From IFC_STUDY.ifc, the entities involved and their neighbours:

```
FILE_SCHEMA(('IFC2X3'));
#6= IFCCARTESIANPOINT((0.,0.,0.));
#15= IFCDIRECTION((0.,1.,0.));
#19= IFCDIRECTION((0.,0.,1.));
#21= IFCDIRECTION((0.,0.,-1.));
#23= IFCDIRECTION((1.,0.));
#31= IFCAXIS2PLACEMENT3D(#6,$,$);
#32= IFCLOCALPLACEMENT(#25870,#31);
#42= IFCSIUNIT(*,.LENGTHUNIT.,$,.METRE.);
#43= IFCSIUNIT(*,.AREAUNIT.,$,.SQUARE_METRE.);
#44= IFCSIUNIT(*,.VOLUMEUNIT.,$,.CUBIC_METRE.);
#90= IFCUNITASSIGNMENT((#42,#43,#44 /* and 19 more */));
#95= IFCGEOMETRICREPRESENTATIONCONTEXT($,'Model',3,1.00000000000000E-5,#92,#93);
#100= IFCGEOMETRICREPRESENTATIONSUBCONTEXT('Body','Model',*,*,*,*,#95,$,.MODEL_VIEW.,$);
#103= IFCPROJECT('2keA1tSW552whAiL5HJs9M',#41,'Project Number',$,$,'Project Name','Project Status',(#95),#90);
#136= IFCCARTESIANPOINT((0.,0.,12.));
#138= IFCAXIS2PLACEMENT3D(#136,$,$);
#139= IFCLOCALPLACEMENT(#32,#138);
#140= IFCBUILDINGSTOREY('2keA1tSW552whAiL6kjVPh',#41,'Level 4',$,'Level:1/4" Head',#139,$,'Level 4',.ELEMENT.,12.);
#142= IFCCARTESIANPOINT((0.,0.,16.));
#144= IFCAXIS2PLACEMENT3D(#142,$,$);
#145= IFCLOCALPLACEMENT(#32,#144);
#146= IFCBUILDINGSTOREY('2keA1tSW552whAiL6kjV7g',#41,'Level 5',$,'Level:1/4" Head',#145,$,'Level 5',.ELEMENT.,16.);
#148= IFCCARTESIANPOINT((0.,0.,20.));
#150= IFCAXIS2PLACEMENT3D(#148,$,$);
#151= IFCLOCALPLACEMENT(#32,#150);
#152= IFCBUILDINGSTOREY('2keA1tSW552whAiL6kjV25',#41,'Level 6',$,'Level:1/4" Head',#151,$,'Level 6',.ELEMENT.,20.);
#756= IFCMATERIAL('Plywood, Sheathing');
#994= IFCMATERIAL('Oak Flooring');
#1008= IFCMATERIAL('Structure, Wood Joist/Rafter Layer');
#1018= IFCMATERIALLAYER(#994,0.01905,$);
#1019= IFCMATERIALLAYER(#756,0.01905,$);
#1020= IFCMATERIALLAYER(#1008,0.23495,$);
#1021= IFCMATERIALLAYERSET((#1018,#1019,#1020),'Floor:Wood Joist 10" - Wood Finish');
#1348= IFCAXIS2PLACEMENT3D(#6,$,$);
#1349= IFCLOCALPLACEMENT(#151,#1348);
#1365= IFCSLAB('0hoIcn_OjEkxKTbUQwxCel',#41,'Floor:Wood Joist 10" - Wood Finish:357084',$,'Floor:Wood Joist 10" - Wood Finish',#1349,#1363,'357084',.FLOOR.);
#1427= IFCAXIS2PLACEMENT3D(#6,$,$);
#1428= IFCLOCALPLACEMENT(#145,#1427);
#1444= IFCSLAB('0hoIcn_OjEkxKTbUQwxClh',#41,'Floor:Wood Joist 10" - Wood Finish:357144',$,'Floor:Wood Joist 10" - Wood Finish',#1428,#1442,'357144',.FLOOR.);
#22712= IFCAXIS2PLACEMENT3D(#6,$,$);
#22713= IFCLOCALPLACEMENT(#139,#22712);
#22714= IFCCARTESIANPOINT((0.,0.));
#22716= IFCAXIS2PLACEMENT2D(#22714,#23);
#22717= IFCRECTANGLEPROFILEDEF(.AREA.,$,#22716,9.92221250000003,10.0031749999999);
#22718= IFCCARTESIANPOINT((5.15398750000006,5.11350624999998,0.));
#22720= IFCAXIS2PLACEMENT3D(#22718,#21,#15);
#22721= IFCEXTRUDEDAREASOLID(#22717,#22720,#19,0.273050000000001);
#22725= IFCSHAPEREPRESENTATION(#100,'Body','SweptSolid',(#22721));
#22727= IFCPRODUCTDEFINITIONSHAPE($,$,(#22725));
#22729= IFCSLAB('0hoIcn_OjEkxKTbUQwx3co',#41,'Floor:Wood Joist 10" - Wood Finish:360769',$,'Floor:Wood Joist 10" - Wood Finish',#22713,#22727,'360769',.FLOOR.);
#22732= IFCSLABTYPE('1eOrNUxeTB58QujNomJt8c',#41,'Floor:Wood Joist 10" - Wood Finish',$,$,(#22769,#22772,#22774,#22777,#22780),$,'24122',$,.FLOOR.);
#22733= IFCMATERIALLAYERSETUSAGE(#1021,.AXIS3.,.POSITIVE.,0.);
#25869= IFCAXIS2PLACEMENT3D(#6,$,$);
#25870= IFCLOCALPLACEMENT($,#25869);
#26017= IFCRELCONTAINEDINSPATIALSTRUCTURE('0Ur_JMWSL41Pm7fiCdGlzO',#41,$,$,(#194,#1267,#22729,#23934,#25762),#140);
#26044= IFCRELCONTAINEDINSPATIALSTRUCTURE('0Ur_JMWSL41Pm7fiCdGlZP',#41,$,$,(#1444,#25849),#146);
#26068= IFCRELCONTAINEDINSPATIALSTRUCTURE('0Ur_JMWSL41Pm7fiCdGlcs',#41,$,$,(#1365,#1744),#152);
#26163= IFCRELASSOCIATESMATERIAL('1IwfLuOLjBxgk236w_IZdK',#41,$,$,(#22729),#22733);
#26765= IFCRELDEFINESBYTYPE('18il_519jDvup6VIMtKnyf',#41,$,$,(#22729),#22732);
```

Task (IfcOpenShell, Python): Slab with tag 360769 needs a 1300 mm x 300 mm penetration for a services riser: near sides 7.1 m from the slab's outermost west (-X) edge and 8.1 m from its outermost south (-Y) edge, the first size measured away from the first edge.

```python
import numpy as np
import ifcopenshell
import ifcopenshell.api.feature
import ifcopenshell.api.geometry
import ifcopenshell.api.root
import ifcopenshell.geom
import ifcopenshell.util.placement
import ifcopenshell.util.representation
import ifcopenshell.util.shape
import ifcopenshell.util.unit

model = ifcopenshell.open("IFC_STUDY.ifc")
unit_scale = ifcopenshell.util.unit.calculate_unit_scale(model)
settings = ifcopenshell.geom.settings()


def volume(element):
    """Net volume in cubic metres, openings subtracted."""
    shape = ifcopenshell.geom.create_shape(settings, element)
    return ifcopenshell.util.shape.get_volume(shape.geometry)


slab = model.by_id(22729)
before = volume(slab)

# Extent in the slab's own axes, in metres. The edges named are its -X and -Y sides.
slab_shape = ifcopenshell.geom.create_shape(settings, slab)
vertices = ifcopenshell.util.shape.get_vertices(slab_shape.geometry)
x_min, y_min, bottom = vertices.min(axis=0)
top = vertices[:, 2].max()

opening = ifcopenshell.api.root.create_entity(model, ifc_class="IfcOpeningElement", name="Services riser opening")
context = ifcopenshell.util.representation.get_context(model, "Model", "Body", "MODEL_VIEW")
width, depth = 1.3, 0.3
outline = [(0.0, 0.0), (width, 0.0), (width, depth), (0.0, depth), (0.0, 0.0)]
# Overshoot both faces by 50 mm so the cut is clean.
shape = ifcopenshell.api.geometry.add_slab_representation(
    model, context=context, depth=top - bottom + 0.1, polyline=outline
)
ifcopenshell.api.geometry.assign_representation(model, product=opening, representation=shape)

matrix = ifcopenshell.util.placement.get_local_placement(slab.ObjectPlacement)
matrix[:, 3] = matrix @ np.append(np.array([x_min + 7.1, y_min + 8.1, bottom - 0.05]) / unit_scale, 1.0)
ifcopenshell.api.geometry.edit_object_placement(model, product=opening, matrix=matrix, is_si=False)
ifcopenshell.api.feature.add_feature(model, feature=opening, element=slab)

after = volume(slab)

print(f"slab volume {before:.3f} -> {after:.3f} m3")

model.write("IFC_STUDY_rev.ifc")
```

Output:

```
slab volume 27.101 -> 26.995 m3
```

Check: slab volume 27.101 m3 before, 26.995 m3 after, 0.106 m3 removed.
